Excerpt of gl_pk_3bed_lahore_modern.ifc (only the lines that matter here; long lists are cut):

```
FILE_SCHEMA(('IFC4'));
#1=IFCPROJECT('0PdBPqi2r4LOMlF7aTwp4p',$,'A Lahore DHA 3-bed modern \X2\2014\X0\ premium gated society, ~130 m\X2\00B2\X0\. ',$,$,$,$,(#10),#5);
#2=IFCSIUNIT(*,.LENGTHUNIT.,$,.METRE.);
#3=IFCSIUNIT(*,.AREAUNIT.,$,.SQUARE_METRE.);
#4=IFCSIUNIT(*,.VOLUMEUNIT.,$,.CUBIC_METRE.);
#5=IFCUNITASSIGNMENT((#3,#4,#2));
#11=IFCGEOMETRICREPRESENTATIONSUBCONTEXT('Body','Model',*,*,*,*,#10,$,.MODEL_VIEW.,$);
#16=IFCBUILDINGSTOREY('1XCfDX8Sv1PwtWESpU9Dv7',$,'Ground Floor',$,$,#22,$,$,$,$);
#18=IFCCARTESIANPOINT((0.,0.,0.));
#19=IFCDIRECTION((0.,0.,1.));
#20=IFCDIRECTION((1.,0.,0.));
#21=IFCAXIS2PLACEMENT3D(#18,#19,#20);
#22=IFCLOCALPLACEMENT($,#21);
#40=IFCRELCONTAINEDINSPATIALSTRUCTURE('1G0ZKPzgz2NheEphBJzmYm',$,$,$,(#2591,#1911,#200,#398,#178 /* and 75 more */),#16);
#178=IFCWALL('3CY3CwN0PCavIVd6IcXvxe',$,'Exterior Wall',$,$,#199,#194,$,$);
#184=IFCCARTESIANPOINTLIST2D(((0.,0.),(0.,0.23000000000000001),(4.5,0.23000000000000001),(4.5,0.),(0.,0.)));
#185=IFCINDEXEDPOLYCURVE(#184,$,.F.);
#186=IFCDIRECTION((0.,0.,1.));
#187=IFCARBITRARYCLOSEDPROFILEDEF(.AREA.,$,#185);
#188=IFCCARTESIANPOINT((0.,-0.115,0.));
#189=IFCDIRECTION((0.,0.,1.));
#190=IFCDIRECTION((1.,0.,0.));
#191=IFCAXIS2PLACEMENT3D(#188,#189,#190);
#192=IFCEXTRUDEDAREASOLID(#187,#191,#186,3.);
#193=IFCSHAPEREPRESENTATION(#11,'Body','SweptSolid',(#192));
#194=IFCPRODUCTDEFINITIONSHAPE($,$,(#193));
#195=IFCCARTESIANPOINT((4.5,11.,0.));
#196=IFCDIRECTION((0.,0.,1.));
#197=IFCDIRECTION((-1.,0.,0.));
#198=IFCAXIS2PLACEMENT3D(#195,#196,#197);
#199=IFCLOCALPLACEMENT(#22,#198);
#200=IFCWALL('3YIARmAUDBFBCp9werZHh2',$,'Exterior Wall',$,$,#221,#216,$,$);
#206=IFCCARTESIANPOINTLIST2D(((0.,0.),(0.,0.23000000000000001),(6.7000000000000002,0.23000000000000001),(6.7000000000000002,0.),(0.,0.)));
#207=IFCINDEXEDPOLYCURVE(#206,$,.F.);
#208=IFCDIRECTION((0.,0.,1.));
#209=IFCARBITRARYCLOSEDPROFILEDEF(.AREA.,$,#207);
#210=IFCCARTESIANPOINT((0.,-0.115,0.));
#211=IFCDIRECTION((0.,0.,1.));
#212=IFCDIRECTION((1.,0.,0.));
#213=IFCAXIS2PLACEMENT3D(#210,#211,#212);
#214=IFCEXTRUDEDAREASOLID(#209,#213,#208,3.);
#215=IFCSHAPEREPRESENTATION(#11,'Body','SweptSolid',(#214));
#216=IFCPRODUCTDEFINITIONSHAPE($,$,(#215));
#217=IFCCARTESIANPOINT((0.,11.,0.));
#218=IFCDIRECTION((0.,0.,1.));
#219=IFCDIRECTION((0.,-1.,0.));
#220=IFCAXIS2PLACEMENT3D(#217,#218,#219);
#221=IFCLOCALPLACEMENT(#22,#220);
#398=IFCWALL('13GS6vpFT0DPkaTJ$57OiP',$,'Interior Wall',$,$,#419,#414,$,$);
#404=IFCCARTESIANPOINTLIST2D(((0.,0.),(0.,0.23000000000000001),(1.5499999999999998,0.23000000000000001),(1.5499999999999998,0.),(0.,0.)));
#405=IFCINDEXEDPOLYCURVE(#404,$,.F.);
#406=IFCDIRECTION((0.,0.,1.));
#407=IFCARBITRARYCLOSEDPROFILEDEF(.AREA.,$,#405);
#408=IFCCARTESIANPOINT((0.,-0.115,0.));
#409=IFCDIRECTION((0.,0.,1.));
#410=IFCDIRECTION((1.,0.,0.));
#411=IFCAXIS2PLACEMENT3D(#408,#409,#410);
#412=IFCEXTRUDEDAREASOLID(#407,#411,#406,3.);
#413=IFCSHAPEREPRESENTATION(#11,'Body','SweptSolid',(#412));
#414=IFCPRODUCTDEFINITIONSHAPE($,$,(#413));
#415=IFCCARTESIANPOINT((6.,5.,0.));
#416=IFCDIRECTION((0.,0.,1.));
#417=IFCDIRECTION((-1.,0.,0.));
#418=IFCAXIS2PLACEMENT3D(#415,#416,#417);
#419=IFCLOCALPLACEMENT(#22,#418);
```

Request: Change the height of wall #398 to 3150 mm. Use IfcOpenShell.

```python
import ifcopenshell
import ifcopenshell.geom
import ifcopenshell.util.representation
import ifcopenshell.util.shape
import ifcopenshell.util.unit

model = ifcopenshell.open("gl_pk_3bed_lahore_modern.ifc")
unit_scale = ifcopenshell.util.unit.calculate_unit_scale(model)
settings = ifcopenshell.geom.settings()


def volume(element):
    """Net volume in cubic metres, openings subtracted."""
    shape = ifcopenshell.geom.create_shape(settings, element)
    return ifcopenshell.util.shape.get_volume(shape.geometry)


wall = model.by_guid("13GS6vpFT0DPkaTJ$57OiP")
before = volume(wall)

body = ifcopenshell.util.representation.get_representation(wall, "Model", "Body")
solid = body.Items[0]
old_height = solid.Depth
solid.Depth = 3.15 / unit_scale
after = volume(wall)

print(f"height {old_height:g} -> {solid.Depth:g}, volume {before:.3f} -> {after:.3f} m3")

model.write("gl_pk_3bed_lahore_modern_v2.ifc")
```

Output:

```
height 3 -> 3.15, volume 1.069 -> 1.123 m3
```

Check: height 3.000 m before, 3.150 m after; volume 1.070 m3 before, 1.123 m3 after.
